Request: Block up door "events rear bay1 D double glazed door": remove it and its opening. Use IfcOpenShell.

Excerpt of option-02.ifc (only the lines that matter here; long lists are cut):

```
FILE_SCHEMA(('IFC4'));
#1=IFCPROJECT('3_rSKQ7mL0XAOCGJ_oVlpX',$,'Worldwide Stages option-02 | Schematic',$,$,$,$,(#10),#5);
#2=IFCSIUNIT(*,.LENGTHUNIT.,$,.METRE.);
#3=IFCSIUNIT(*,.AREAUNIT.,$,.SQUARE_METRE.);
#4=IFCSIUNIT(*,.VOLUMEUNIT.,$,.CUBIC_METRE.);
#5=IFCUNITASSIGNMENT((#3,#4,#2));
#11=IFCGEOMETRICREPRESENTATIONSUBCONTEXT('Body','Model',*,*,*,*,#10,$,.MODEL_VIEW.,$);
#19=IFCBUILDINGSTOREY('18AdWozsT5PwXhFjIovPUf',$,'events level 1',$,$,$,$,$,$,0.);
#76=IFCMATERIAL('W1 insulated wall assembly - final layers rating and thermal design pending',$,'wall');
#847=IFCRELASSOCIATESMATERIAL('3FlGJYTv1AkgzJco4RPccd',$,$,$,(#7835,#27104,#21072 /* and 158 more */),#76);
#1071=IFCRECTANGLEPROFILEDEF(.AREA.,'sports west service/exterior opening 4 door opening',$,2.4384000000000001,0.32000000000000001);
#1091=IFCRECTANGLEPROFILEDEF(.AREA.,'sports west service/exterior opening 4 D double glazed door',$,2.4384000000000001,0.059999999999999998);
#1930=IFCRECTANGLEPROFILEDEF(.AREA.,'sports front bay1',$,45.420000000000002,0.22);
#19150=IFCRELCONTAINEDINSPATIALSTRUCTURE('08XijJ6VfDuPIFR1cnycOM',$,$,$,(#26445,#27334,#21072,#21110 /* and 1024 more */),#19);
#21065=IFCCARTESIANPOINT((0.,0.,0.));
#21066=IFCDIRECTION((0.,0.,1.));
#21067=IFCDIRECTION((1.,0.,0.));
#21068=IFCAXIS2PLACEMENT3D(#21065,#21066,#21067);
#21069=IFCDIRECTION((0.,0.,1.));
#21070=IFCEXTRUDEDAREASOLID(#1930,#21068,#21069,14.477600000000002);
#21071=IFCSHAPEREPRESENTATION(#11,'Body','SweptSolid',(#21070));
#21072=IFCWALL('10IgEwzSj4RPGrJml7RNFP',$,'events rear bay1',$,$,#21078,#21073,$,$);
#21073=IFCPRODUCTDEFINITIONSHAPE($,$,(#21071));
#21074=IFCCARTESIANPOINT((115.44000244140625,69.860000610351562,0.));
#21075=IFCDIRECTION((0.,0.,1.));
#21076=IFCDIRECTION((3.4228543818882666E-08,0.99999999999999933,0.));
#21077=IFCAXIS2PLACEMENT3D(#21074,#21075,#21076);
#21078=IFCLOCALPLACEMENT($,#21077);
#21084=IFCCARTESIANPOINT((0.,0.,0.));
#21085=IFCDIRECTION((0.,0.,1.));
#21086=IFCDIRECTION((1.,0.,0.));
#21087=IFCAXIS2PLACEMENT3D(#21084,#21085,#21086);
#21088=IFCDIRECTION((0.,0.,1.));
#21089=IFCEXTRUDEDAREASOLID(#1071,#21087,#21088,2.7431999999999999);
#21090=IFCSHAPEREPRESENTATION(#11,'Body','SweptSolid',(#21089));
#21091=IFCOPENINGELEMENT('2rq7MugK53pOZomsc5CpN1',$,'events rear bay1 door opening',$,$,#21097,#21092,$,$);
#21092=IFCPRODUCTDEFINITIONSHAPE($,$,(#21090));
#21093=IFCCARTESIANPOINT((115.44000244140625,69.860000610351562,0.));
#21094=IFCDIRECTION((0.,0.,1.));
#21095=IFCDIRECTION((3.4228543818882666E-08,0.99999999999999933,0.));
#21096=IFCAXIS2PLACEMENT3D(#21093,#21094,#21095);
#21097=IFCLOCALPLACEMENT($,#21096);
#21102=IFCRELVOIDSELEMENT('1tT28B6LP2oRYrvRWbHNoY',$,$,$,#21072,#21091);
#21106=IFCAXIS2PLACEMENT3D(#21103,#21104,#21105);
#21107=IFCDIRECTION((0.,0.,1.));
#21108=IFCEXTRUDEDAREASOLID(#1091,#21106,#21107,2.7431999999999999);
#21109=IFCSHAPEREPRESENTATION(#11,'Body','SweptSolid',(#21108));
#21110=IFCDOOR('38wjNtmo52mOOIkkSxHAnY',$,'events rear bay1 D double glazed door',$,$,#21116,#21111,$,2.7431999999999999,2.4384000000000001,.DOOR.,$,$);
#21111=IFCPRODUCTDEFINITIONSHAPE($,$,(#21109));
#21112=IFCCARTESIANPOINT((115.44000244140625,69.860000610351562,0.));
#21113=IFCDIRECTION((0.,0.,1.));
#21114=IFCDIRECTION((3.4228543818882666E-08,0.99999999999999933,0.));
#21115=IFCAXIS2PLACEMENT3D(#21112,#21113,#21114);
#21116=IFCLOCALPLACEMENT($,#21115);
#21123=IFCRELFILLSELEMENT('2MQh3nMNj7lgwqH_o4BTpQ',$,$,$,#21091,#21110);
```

```python
import ifcopenshell
import ifcopenshell.api.feature
import ifcopenshell.api.root
import ifcopenshell.geom
import ifcopenshell.util.shape

model = ifcopenshell.open("option-02.ifc")
settings = ifcopenshell.geom.settings()


def volume(element):
    """Net volume in cubic metres, openings subtracted."""
    shape = ifcopenshell.geom.create_shape(settings, element)
    return ifcopenshell.util.shape.get_volume(shape.geometry)


door = model.by_guid("38wjNtmo52mOOIkkSxHAnY")
opening = door.FillsVoids[0].RelatingOpeningElement
wall = opening.VoidsElements[0].RelatingBuildingElement
before = volume(wall)

ifcopenshell.api.root.remove_product(model, product=door)
ifcopenshell.api.feature.remove_feature(model, feature=opening)

after = volume(wall)

print(f"wall volume {before:.3f} -> {after:.3f} m3")

model.write("option-02_updated.ifc")
```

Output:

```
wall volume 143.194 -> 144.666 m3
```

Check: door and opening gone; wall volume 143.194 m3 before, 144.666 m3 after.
